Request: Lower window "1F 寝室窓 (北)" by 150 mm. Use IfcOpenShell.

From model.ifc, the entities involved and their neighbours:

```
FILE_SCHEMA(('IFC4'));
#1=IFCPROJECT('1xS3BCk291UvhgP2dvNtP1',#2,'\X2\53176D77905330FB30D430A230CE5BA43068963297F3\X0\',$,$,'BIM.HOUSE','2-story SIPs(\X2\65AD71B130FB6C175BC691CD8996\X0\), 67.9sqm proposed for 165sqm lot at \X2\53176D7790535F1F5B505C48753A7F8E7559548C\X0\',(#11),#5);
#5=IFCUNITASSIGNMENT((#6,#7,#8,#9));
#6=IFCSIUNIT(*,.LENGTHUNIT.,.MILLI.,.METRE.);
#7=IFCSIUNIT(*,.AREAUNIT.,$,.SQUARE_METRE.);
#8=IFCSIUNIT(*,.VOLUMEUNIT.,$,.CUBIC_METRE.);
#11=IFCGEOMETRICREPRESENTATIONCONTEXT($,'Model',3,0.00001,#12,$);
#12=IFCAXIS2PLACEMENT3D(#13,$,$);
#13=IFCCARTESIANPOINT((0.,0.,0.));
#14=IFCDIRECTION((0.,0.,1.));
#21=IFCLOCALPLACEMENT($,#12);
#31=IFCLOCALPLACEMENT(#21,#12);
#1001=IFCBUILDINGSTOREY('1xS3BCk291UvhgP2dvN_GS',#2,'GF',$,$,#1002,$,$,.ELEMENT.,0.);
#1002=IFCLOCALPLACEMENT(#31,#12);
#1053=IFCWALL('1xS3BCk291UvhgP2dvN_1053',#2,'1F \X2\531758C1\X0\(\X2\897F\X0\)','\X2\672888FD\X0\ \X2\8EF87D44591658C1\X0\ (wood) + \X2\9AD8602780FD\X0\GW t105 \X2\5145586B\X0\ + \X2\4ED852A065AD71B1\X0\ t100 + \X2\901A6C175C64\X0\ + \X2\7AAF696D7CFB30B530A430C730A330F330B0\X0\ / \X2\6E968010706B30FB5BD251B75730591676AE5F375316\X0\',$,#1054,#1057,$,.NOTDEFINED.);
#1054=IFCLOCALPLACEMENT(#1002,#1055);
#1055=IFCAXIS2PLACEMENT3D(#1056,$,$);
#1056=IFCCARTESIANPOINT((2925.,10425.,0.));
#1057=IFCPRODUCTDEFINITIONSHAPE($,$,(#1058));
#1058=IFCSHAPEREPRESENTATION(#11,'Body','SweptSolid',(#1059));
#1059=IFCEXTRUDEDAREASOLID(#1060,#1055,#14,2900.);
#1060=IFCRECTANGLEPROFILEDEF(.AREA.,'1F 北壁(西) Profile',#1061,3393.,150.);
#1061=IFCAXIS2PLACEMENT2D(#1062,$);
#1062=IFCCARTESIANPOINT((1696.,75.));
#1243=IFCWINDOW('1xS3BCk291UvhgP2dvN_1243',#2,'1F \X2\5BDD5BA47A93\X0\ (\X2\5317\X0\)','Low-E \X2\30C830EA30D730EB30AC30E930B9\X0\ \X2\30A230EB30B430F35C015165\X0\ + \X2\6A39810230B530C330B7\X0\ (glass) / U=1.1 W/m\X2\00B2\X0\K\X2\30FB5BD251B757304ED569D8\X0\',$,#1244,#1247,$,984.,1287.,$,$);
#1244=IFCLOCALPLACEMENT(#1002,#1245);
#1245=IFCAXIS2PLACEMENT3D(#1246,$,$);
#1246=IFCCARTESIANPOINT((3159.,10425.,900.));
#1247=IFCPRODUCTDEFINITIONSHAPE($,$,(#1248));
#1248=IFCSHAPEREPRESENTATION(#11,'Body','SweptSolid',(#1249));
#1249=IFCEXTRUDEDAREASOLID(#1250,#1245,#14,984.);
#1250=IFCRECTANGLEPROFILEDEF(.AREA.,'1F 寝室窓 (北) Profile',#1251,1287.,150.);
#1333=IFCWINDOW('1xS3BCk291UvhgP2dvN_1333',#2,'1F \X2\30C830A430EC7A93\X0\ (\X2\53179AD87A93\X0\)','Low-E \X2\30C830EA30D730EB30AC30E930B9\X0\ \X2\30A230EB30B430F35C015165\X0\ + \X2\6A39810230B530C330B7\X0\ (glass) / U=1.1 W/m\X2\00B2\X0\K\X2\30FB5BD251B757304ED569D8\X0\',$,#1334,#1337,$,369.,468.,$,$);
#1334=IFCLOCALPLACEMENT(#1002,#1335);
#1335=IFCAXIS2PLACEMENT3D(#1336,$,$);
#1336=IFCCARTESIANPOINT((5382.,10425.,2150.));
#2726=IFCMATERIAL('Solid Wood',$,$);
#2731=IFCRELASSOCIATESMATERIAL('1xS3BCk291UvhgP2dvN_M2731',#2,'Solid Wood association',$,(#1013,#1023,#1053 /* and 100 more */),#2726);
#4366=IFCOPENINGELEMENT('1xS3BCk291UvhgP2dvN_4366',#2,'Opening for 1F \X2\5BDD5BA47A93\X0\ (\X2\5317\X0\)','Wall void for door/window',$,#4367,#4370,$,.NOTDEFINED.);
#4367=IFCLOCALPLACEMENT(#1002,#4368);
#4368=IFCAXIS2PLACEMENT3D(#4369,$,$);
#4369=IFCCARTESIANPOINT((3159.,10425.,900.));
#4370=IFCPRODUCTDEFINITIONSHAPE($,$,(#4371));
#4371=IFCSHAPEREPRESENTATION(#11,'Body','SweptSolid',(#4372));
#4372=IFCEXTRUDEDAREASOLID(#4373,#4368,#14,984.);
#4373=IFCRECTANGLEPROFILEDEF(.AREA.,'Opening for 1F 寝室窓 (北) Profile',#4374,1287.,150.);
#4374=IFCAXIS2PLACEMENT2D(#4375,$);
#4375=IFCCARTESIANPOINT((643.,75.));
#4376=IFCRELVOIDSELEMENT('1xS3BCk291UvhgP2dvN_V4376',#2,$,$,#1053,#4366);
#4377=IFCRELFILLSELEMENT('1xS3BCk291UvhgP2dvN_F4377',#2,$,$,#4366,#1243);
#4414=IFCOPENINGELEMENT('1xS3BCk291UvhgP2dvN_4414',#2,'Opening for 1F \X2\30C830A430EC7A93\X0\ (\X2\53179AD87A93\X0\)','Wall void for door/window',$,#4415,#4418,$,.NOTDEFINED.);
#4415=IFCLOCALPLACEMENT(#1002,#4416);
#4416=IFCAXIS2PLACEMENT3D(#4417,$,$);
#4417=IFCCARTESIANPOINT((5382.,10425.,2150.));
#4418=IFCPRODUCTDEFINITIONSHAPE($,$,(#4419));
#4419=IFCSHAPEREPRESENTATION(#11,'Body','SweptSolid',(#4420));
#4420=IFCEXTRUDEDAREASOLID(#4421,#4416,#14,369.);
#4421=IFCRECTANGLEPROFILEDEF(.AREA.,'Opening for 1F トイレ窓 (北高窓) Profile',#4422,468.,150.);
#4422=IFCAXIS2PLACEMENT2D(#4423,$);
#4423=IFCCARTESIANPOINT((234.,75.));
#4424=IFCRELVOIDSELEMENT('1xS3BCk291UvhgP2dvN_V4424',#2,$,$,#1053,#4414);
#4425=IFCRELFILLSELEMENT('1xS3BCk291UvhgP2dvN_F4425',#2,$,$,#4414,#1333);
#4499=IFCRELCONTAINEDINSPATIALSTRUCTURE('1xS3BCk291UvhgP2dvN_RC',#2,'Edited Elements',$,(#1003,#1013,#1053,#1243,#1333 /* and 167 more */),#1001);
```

```python
import numpy as np
import ifcopenshell
import ifcopenshell.api.geometry
import ifcopenshell.util.placement
import ifcopenshell.util.unit

model = ifcopenshell.open("model.ifc")
unit_scale = ifcopenshell.util.unit.calculate_unit_scale(model)

window = model.by_id(1243)
opening = window.FillsVoids[0].RelatingOpeningElement
dz = -150.0

shift = np.array([0.0, 0.0, dz])
# The window is not placed relative to its opening, so move both.
for product in (opening, window):
    matrix = ifcopenshell.util.placement.get_local_placement(product.ObjectPlacement)
    matrix[:3, 3] += shift
    ifcopenshell.api.geometry.edit_object_placement(model, product=product, matrix=matrix, is_si=False)

print(f"moved by {dz * unit_scale:+.3f} m")

model.write("model-out.ifc")
```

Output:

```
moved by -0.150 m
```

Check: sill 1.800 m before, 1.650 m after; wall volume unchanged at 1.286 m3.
